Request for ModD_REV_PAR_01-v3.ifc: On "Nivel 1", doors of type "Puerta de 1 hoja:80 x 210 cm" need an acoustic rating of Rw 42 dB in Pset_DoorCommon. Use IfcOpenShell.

First a look at what the model holds.

```python
import ifcopenshell
import ifcopenshell.util.element

model = ifcopenshell.open("ModD_REV_PAR_01-v3.ifc")
print(model.schema)
storey = next(s for s in model.by_type("IfcBuildingStorey") if s.Name == "Nivel 1")
doors = [e for e in ifcopenshell.util.element.get_decomposition(storey) if e.is_a("IfcDoor")]
seen = {}
for e in doors:
    element_type = ifcopenshell.util.element.get_type(e)
    key = (element_type.Name if element_type != e and element_type else None, ifcopenshell.util.element.get_pset(e, "Pset_DoorCommon", "AcousticRating"))
    seen[key] = seen.get(key, 0) + 1
for (name, value), count in sorted(seen.items(), key=str):
    print(count, "x", name, "|", value)
```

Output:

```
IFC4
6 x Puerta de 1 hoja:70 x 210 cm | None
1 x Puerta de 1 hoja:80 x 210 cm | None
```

```python
import ifcopenshell
import ifcopenshell.api.pset
import ifcopenshell.util.element

model = ifcopenshell.open("ModD_REV_PAR_01-v3.ifc")

storey = next(s for s in model.by_type("IfcBuildingStorey") if s.Name == "Nivel 1")
doors = [e for e in ifcopenshell.util.element.get_decomposition(storey) if e.is_a("IfcDoor")]

count = 0
for e in doors:
    element_type = ifcopenshell.util.element.get_type(e)
    if element_type in (None, e) or element_type.Name != "Puerta de 1 hoja:80 x 210 cm":
        continue
    # add_pset returns the element's existing set when there is one.
    pset = ifcopenshell.api.pset.add_pset(model, product=e, name="Pset_DoorCommon")
    ifcopenshell.api.pset.edit_pset(model, pset=pset, properties={"AcousticRating": "Rw 42 dB"})
    count += 1

print(count, "doors updated")

model.write("ModD_REV_PAR_01-v3_edited.ifc")
```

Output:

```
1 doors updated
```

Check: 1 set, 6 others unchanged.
